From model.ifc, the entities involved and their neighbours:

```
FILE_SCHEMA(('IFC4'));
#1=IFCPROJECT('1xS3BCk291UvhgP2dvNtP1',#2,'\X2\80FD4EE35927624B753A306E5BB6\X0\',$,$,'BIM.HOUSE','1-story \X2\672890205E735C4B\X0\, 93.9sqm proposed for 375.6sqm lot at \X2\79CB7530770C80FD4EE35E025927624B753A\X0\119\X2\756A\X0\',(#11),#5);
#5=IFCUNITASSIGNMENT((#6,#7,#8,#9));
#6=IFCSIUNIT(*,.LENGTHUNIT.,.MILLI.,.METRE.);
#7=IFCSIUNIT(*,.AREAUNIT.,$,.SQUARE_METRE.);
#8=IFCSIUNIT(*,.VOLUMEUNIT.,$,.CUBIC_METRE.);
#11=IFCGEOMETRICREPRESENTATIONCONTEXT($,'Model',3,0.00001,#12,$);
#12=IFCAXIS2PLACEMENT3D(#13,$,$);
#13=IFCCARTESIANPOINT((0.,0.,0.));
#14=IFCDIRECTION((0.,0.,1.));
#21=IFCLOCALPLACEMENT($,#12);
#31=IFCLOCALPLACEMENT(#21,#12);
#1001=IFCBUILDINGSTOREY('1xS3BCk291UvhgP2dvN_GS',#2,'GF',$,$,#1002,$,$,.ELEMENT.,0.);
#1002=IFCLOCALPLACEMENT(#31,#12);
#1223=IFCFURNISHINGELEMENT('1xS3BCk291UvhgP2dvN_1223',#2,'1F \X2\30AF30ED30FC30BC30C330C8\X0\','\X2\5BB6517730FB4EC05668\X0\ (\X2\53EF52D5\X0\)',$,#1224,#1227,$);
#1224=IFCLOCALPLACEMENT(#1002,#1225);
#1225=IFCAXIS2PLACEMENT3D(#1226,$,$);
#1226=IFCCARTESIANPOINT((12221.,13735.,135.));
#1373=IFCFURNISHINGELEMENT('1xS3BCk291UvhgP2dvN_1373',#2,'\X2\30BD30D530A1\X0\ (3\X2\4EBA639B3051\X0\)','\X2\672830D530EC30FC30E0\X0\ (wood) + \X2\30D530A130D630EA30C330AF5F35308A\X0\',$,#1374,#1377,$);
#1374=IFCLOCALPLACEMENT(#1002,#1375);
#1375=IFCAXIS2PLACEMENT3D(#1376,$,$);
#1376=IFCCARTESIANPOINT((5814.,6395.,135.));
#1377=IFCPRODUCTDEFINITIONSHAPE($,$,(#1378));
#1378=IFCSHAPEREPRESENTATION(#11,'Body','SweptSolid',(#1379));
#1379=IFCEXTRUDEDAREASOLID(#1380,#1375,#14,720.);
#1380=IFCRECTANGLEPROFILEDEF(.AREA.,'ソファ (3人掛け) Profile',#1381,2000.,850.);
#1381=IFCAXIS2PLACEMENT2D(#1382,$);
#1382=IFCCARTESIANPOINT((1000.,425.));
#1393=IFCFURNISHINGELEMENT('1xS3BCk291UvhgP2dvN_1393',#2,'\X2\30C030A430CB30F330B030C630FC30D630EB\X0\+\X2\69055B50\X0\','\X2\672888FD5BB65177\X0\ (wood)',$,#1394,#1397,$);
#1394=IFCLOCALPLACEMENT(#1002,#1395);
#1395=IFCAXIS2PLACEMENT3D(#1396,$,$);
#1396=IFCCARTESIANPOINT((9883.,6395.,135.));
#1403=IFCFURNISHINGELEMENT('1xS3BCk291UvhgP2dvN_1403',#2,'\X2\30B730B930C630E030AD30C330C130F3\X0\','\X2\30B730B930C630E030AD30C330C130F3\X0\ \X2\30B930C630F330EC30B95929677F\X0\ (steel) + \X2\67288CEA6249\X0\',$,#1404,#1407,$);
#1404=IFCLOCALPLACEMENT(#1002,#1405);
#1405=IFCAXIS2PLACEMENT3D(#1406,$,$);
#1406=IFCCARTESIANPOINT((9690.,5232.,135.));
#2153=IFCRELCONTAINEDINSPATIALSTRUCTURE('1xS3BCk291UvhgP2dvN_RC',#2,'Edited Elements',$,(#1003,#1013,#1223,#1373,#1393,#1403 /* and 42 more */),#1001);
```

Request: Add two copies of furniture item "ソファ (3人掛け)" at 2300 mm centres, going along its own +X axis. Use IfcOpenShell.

```python
import ifcopenshell
import ifcopenshell.api.geometry
import ifcopenshell.api.root
import ifcopenshell.util.element
import ifcopenshell.util.placement
import ifcopenshell.util.unit

model = ifcopenshell.open("model.ifc")
unit_scale = ifcopenshell.util.unit.calculate_unit_scale(model)


def reuse_history(source, copy):
    """copy_class also copies each property set's owner history, people and application; keep the originals."""
    for rel in copy.IsDefinedBy:
        if rel.is_a("IfcRelDefinesByProperties") and (history := rel.RelatingPropertyDefinition.OwnerHistory):
            rel.RelatingPropertyDefinition.OwnerHistory = source.OwnerHistory
            ifcopenshell.util.element.remove_deep2(model, history)


source = model.by_guid("1xS3BCk291UvhgP2dvN_1373")
base = ifcopenshell.util.placement.get_local_placement(source.ObjectPlacement)
step = base[:3, 0] * 2.3 / unit_scale

for i in range(1, 3):
    copy = ifcopenshell.api.root.copy_class(model, product=source)
    copy.Representation = ifcopenshell.util.element.copy_deep(
        model, source.Representation, exclude=["IfcGeometricRepresentationContext", "IfcRepresentationMap"]
    )
    reuse_history(source, copy)
    matrix = base.copy()
    matrix[:3, 3] += i * step
    print("added at", matrix[:3, 3].round(3) + 0.0)
    ifcopenshell.api.geometry.edit_object_placement(model, product=copy, matrix=matrix, is_si=False)

model.write("model-out.ifc")
```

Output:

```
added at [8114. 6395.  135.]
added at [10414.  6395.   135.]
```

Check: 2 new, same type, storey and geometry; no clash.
